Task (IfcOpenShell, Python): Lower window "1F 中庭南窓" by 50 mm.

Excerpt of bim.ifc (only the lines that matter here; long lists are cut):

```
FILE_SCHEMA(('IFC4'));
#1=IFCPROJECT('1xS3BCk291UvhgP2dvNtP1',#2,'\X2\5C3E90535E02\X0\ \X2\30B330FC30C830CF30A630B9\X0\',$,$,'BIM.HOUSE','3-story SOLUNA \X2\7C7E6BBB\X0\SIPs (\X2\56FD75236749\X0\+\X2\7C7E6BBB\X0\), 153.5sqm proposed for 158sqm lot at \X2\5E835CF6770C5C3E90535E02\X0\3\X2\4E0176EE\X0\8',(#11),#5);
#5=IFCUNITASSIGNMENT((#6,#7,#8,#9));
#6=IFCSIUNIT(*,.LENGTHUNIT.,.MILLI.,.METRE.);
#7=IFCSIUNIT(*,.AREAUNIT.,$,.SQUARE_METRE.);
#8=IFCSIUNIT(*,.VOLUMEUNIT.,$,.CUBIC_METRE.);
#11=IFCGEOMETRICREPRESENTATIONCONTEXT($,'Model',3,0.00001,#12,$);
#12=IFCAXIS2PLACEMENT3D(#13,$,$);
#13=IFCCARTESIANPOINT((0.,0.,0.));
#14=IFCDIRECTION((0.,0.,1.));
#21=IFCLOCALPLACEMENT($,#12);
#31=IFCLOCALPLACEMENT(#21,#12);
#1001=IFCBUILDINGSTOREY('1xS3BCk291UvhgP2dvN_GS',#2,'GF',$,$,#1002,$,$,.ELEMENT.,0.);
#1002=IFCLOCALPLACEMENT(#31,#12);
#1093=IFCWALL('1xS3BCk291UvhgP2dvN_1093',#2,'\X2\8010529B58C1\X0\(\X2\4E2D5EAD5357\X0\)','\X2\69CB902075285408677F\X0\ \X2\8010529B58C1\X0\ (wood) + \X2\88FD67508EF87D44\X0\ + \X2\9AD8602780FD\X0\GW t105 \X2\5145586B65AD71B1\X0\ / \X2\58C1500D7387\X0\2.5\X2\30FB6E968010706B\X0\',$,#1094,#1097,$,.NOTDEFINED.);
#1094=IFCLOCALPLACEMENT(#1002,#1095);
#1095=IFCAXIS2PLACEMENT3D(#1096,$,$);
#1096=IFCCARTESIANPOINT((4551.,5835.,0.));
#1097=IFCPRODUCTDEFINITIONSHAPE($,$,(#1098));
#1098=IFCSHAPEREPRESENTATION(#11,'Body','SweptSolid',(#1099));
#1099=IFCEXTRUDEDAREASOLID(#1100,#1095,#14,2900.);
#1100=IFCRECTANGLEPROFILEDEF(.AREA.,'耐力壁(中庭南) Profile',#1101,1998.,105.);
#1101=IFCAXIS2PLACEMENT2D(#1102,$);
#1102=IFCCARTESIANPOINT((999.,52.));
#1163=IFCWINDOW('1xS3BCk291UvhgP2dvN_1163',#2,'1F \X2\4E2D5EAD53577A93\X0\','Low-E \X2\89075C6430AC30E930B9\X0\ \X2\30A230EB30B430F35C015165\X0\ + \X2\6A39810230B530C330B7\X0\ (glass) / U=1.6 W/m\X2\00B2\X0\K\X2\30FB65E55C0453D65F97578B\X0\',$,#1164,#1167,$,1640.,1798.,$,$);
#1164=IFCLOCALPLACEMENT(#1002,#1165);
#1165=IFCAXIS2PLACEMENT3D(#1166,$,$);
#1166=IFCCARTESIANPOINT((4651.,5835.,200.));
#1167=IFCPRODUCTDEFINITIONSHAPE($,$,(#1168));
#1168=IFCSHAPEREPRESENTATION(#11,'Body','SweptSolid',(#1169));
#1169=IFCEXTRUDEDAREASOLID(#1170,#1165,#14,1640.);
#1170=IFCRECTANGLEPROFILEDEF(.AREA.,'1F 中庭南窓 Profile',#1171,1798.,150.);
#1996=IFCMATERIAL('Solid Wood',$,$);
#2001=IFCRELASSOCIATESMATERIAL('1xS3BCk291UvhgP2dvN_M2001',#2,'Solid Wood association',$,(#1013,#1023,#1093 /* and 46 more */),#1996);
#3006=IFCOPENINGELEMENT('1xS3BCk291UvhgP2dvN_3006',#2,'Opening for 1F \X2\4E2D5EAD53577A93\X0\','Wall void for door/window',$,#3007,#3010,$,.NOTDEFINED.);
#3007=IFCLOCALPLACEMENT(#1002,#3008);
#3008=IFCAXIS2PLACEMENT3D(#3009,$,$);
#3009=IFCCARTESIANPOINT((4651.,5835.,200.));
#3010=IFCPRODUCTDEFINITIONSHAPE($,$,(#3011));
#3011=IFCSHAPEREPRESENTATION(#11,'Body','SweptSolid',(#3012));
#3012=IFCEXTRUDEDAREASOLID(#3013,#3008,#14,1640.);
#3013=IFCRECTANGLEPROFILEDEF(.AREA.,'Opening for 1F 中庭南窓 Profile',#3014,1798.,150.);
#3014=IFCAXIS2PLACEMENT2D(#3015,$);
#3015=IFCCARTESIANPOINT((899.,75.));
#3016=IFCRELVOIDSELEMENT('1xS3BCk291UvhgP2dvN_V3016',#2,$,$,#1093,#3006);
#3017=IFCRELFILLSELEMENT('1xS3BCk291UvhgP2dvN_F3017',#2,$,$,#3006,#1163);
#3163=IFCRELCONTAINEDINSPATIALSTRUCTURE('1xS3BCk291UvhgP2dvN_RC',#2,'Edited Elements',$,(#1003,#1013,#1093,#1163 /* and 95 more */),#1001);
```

```python
import numpy as np
import ifcopenshell
import ifcopenshell.api.geometry
import ifcopenshell.util.placement
import ifcopenshell.util.unit

model = ifcopenshell.open("bim.ifc")
unit_scale = ifcopenshell.util.unit.calculate_unit_scale(model)

window = model.by_id(1163)
opening = window.FillsVoids[0].RelatingOpeningElement
dz = -0.05 / unit_scale

shift = np.array([0.0, 0.0, dz])
# The window is not placed relative to its opening, so move both.
for product in (opening, window):
    matrix = ifcopenshell.util.placement.get_local_placement(product.ObjectPlacement)
    matrix[:3, 3] += shift
    ifcopenshell.api.geometry.edit_object_placement(model, product=product, matrix=matrix, is_si=False)

print(f"moved by {dz * unit_scale:+.3f} m")

model.write("bim-out.ifc")
```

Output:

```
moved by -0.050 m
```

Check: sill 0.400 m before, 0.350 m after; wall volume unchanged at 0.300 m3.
